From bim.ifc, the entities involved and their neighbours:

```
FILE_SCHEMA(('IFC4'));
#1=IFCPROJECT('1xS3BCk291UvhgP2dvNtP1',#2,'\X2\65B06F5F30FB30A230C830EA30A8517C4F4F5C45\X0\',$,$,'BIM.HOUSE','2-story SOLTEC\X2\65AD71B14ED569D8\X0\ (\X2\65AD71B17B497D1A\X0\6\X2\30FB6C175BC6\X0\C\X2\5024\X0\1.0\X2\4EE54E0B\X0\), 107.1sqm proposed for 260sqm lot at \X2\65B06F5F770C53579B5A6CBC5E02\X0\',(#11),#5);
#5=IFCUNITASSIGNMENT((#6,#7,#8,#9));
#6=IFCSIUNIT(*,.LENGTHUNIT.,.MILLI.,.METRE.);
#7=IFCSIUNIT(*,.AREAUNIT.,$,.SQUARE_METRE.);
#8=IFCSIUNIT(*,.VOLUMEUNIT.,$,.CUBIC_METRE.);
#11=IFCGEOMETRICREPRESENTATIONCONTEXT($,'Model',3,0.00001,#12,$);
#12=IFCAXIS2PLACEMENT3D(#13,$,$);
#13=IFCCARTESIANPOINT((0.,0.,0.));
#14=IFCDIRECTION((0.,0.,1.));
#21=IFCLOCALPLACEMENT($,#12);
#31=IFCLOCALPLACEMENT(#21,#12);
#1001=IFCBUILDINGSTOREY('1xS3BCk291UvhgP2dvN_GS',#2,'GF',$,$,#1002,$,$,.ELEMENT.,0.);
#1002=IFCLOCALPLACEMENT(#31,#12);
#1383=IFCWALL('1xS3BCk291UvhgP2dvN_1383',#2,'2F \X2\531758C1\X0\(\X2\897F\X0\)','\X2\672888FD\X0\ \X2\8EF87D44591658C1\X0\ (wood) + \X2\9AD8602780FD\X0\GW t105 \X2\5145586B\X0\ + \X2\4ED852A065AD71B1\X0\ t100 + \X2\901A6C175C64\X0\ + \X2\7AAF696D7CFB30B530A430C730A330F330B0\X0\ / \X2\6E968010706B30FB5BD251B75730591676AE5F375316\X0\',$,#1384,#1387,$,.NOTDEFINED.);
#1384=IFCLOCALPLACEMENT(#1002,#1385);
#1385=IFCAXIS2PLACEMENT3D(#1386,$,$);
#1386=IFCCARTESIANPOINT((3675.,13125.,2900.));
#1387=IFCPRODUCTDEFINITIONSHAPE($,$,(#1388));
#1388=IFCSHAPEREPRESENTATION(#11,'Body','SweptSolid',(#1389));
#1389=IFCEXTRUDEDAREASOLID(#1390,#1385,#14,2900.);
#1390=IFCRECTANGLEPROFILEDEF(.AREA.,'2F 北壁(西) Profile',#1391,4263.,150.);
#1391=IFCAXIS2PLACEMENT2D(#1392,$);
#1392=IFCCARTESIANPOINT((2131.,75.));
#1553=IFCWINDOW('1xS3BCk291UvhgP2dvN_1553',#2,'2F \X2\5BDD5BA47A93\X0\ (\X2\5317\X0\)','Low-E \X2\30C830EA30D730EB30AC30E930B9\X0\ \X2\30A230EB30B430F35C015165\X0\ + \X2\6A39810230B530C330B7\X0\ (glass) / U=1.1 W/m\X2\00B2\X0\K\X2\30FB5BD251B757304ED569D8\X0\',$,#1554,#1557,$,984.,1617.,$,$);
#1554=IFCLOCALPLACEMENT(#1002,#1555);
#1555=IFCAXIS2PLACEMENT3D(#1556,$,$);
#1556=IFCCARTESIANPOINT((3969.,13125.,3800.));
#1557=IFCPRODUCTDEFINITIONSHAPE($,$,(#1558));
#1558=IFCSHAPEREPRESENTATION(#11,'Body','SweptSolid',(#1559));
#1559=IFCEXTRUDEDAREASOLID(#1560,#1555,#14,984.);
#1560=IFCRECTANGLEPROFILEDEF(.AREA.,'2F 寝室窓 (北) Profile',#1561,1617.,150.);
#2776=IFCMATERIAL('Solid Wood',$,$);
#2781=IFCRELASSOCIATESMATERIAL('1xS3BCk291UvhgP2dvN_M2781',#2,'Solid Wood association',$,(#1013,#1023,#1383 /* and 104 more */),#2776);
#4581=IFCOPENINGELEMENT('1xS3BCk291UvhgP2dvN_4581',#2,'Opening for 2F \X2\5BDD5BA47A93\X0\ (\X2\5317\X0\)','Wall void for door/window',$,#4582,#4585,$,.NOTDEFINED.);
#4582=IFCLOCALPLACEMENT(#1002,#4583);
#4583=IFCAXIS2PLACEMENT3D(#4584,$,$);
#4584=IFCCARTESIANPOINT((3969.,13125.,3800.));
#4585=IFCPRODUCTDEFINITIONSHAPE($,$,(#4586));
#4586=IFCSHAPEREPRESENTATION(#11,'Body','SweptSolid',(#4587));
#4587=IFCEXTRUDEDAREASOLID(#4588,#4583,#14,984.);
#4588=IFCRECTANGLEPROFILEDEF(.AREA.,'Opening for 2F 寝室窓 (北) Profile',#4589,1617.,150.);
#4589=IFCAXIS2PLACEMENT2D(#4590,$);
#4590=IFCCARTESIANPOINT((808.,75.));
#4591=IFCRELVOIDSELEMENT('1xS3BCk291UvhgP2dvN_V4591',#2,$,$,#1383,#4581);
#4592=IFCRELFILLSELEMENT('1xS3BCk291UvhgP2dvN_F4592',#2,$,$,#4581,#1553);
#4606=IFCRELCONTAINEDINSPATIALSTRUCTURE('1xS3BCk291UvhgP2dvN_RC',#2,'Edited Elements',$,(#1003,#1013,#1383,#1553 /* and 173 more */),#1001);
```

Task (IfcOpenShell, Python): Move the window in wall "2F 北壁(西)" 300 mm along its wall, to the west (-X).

```python
import ifcopenshell
import ifcopenshell.api.geometry
import ifcopenshell.util.placement
import ifcopenshell.util.unit

model = ifcopenshell.open("bim.ifc")
unit_scale = ifcopenshell.util.unit.calculate_unit_scale(model)

window = model.by_guid("1xS3BCk291UvhgP2dvN_1553")
opening = window.FillsVoids[0].RelatingOpeningElement
wall = opening.VoidsElements[0].RelatingBuildingElement

wall_matrix = ifcopenshell.util.placement.get_local_placement(wall.ObjectPlacement)
shift = wall_matrix[:3, 0] * -0.3 / unit_scale
before = ifcopenshell.util.placement.get_local_placement(window.ObjectPlacement)[:3, 3].copy()

# The window is not placed relative to its opening, so move both.
for product in (opening, window):
    matrix = ifcopenshell.util.placement.get_local_placement(product.ObjectPlacement)
    matrix[:3, 3] += shift
    ifcopenshell.api.geometry.edit_object_placement(model, product=product, matrix=matrix, is_si=False)

after = ifcopenshell.util.placement.get_local_placement(window.ObjectPlacement)[:3, 3]
print("window moved by", (after - before).round(3) + 0.0)

model.write("bim-out.ifc")
```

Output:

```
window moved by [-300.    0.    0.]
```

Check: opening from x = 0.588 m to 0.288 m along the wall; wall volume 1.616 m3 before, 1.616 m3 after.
